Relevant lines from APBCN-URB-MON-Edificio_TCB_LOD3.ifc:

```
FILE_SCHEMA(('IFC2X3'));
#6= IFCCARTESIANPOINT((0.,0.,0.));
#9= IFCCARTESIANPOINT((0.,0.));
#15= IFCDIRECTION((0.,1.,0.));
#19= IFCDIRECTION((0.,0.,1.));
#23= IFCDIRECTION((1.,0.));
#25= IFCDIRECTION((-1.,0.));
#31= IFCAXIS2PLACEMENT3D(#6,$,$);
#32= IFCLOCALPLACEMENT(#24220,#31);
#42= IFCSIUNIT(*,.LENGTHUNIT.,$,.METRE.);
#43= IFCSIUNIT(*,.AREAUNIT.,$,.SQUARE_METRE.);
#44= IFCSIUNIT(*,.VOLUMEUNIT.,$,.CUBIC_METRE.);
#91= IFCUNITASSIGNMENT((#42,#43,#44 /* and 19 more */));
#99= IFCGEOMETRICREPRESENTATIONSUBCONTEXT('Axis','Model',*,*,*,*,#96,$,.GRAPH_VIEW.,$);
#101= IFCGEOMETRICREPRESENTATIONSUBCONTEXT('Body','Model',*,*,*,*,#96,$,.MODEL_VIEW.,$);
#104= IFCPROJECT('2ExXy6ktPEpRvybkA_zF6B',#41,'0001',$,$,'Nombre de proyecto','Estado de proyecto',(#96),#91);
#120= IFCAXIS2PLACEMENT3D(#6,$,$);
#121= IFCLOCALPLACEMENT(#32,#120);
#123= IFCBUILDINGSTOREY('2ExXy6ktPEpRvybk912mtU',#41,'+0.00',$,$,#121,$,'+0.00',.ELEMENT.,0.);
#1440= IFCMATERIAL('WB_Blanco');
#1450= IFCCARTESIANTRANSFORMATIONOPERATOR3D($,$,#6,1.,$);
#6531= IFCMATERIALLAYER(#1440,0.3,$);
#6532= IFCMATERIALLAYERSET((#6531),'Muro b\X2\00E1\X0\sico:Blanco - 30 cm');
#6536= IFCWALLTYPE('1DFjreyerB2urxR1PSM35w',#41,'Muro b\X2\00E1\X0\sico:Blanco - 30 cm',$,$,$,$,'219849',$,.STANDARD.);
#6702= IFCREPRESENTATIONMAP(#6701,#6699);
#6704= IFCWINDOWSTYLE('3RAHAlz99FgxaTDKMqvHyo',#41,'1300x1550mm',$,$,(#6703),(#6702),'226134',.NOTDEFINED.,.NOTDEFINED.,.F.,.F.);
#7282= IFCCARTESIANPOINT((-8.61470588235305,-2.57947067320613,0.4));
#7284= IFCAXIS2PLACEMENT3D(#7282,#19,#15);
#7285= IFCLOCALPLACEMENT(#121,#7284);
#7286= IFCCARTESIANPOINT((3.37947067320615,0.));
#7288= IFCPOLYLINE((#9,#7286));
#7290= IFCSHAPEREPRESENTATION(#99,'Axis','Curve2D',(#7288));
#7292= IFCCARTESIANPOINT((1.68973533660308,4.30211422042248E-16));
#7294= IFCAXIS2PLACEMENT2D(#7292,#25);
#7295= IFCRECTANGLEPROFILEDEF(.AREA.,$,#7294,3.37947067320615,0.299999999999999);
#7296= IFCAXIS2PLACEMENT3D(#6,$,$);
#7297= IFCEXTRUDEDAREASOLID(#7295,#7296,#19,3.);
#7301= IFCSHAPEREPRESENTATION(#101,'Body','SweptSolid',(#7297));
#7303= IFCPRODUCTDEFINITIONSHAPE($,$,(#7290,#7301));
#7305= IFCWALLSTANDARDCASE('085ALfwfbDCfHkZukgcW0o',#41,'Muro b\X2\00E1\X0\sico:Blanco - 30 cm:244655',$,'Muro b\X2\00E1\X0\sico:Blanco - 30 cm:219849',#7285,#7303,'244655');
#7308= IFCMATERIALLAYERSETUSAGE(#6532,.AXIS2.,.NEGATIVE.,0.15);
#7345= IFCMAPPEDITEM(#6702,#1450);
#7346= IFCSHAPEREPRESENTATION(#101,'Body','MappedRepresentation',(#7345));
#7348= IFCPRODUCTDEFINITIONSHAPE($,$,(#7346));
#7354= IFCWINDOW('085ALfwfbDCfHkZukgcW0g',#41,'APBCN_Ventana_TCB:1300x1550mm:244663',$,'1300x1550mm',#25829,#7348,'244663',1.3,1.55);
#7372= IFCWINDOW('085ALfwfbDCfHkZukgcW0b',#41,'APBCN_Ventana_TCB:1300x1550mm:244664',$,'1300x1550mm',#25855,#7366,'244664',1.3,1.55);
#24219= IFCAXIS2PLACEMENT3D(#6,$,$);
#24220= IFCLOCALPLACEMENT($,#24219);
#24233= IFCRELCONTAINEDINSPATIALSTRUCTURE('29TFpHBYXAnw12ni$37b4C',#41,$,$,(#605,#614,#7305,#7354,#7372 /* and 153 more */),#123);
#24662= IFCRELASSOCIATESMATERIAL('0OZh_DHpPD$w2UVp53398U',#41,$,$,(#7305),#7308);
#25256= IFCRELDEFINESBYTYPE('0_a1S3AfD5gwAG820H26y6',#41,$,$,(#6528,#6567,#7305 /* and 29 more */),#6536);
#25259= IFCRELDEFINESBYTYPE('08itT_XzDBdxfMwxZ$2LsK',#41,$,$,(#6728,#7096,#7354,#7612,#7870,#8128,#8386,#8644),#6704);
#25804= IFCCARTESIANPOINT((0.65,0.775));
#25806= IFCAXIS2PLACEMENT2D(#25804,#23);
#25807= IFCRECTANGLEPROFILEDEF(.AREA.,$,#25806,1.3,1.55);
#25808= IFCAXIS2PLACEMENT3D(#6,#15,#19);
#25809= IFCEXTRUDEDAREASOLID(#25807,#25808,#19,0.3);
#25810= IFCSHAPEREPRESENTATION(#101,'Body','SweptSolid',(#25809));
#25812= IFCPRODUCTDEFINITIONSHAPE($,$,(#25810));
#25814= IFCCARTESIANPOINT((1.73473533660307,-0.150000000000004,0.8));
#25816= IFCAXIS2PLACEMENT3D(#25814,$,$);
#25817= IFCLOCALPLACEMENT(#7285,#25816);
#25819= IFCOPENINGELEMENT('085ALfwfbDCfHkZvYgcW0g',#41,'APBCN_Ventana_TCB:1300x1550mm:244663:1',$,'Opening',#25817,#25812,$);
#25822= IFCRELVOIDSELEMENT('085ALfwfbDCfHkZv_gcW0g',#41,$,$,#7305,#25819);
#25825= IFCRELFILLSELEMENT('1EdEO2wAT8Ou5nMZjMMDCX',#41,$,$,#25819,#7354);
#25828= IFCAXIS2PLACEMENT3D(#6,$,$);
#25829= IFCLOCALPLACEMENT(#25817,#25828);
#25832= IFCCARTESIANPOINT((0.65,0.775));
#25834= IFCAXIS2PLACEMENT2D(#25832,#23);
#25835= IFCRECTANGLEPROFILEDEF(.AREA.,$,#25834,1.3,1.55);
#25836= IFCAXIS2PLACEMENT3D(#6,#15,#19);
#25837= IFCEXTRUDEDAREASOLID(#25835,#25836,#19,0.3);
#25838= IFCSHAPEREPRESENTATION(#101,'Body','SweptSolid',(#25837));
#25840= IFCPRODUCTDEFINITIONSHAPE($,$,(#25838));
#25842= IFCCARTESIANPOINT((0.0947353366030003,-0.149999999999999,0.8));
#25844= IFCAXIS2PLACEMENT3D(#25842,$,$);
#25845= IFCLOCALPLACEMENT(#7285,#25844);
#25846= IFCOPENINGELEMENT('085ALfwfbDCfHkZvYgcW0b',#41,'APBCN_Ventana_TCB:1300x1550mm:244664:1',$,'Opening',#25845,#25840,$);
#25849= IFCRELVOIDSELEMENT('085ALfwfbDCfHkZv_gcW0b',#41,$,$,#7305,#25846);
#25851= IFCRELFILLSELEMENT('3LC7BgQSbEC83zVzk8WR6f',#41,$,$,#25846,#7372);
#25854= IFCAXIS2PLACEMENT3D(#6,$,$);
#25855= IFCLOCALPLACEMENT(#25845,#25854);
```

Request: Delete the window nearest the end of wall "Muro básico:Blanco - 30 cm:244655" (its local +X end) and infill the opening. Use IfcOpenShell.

```python
import ifcopenshell
import ifcopenshell.api.feature
import ifcopenshell.api.root
import ifcopenshell.geom
import ifcopenshell.util.shape

model = ifcopenshell.open("APBCN-URB-MON-Edificio_TCB_LOD3.ifc")
settings = ifcopenshell.geom.settings()


def volume(element):
    """Net volume in cubic metres, openings subtracted."""
    shape = ifcopenshell.geom.create_shape(settings, element)
    return ifcopenshell.util.shape.get_volume(shape.geometry)


window = model.by_id(7354)
opening = window.FillsVoids[0].RelatingOpeningElement
wall = opening.VoidsElements[0].RelatingBuildingElement
before = volume(wall)

ifcopenshell.api.root.remove_product(model, product=window)
ifcopenshell.api.feature.remove_feature(model, feature=opening)

after = volume(wall)

print(f"wall volume {before:.3f} -> {after:.3f} m3")

model.write("APBCN-URB-MON-Edificio_TCB_LOD3-out.ifc")
```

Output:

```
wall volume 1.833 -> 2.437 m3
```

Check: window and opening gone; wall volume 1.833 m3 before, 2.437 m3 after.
